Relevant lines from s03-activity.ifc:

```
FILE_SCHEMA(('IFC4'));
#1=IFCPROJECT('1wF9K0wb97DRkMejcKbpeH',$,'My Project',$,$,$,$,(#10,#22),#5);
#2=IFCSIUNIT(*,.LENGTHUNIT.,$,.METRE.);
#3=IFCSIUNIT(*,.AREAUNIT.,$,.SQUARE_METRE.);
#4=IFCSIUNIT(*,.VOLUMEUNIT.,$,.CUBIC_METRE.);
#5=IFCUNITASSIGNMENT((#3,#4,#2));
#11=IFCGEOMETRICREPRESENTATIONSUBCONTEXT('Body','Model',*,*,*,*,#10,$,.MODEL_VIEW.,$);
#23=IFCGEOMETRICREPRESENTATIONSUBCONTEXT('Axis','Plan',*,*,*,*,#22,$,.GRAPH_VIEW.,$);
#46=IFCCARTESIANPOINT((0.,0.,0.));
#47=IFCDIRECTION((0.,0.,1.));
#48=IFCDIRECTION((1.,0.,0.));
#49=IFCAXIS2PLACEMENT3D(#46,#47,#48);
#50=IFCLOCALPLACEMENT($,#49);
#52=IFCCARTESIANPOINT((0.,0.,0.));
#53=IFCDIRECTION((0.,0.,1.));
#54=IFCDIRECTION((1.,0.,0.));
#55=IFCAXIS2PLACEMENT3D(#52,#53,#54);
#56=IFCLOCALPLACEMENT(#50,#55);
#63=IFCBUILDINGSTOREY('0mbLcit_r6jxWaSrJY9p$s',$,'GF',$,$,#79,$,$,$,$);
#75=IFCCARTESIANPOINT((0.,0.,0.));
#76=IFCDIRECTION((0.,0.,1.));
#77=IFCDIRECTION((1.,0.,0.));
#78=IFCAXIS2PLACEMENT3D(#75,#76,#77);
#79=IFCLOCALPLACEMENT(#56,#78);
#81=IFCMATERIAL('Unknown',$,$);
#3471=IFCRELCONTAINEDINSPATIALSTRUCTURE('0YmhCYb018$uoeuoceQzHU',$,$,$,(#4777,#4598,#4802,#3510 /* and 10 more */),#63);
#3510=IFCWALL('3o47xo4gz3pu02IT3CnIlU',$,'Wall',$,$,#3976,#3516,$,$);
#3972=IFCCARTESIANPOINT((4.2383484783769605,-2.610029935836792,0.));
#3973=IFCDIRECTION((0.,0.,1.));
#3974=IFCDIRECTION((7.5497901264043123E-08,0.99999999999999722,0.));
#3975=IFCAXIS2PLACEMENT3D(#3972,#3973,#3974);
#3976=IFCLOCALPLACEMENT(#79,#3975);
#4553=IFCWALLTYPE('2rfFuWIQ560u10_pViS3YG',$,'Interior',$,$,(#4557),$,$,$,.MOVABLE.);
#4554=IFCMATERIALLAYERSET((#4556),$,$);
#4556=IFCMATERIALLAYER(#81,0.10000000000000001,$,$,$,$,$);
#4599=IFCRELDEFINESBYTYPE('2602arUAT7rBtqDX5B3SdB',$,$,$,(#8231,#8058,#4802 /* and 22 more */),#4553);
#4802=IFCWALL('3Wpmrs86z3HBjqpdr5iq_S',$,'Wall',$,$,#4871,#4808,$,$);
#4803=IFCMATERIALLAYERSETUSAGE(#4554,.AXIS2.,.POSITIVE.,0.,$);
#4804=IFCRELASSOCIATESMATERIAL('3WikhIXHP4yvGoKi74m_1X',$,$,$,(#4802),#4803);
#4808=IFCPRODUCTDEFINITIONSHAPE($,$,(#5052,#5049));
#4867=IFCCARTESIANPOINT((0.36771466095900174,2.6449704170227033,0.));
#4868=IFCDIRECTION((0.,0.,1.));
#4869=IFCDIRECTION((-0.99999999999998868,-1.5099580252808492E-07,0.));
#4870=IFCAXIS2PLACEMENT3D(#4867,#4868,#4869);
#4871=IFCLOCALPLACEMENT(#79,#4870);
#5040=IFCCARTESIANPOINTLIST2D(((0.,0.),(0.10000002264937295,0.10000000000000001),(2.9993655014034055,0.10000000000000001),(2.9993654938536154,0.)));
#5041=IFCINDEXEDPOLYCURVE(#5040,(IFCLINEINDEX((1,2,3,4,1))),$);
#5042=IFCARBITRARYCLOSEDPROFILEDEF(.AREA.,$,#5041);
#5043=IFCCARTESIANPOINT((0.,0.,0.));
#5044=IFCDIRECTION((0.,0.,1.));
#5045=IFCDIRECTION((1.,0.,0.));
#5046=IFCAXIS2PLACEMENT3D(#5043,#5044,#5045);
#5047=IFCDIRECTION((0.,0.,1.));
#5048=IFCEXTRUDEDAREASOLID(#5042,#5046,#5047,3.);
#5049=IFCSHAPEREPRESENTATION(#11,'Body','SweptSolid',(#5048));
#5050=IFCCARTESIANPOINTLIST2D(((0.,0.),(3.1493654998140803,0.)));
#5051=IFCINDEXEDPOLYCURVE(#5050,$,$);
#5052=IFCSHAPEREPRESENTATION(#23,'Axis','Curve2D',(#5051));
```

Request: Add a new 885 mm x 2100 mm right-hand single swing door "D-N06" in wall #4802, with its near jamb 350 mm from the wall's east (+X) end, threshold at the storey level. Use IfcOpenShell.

```python
import numpy as np
import ifcopenshell
import ifcopenshell.api.feature
import ifcopenshell.api.geometry
import ifcopenshell.api.root
import ifcopenshell.api.spatial
import ifcopenshell.geom
import ifcopenshell.util.element
import ifcopenshell.util.placement
import ifcopenshell.util.representation
import ifcopenshell.util.shape
import ifcopenshell.util.unit

model = ifcopenshell.open("s03-activity.ifc")
unit_scale = ifcopenshell.util.unit.calculate_unit_scale(model)
settings = ifcopenshell.geom.settings()


def volume(element):
    """Net volume in cubic metres, openings subtracted."""
    shape = ifcopenshell.geom.create_shape(settings, element)
    return ifcopenshell.util.shape.get_volume(shape.geometry)


wall = model.by_guid("3Wpmrs86z3HBjqpdr5iq_S")
storey = ifcopenshell.util.element.get_container(wall, ifc_class="IfcBuildingStorey")
context = ifcopenshell.util.representation.get_context(model, "Model", "Body", "MODEL_VIEW")
before = volume(wall)

width, height, from_end, sill = 0.885, 2.1, 0.35, 0.0  # metres

# The wall runs along its own X axis, and the end named is its -X end.
wall_shape = ifcopenshell.geom.create_shape(settings, wall)
x, y, z = ifcopenshell.util.shape.get_vertices(wall_shape.geometry).T
start = x.min() + from_end
face, thickness = float(y.min()), float(y.max() - y.min())
wall_matrix = ifcopenshell.util.placement.get_local_placement(wall.ObjectPlacement)
level = ifcopenshell.util.placement.get_local_placement(storey.ObjectPlacement)[2, 3]


def in_wall(x, y):
    """Placement at x, y metres in the wall's axes, at sill height."""
    matrix = wall_matrix.copy()
    matrix[:, 3] = wall_matrix @ np.array([x / unit_scale, y / unit_scale, 0.0, 1.0])
    matrix[2, 3] = level + sill / unit_scale
    return matrix


# Opening: a box that overshoots both wall faces by 50 mm.
opening = ifcopenshell.api.root.create_entity(model, ifc_class="IfcOpeningElement", predefined_type="OPENING")
box = ifcopenshell.api.geometry.add_wall_representation(
    model, context=context, length=width, height=height, thickness=thickness + 0.1
)
ifcopenshell.api.geometry.assign_representation(model, product=opening, representation=box)
ifcopenshell.api.geometry.edit_object_placement(model, product=opening, matrix=in_wall(start, face - 0.05), is_si=False)
ifcopenshell.api.feature.add_feature(model, feature=opening, element=wall)

door = ifcopenshell.api.root.create_entity(model, ifc_class="IfcDoor", name="D-N06", predefined_type="DOOR")
door.OverallWidth, door.OverallHeight = width / unit_scale, height / unit_scale
door.OperationType = "SINGLE_SWING_RIGHT"
body = ifcopenshell.api.geometry.add_door_representation(
    model,
    context=context,
    overall_width=door.OverallWidth,
    overall_height=door.OverallHeight,
    operation_type="SINGLE_SWING_RIGHT",
    lining_properties={"LiningDepth": thickness / unit_scale, "ThresholdDepth": thickness / unit_scale},
)
ifcopenshell.api.geometry.assign_representation(model, product=door, representation=body)
ifcopenshell.api.spatial.assign_container(model, products=[door], relating_structure=storey)
ifcopenshell.api.feature.add_filling(model, opening=opening, element=door)

# The lining spans the wall, so the door starts at the wall face.
ifcopenshell.api.geometry.edit_object_placement(model, product=door, matrix=in_wall(start, face), is_si=False)

after = volume(wall)

print(f"wall volume {before:.3f} -> {after:.3f} m3")

model.write("s03-activity-out.ifc")
```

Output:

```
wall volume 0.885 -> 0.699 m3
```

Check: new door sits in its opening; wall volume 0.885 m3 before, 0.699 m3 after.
